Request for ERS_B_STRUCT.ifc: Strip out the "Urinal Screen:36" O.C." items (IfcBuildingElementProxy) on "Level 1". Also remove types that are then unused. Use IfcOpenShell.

First a look at what the model holds.

```python
import ifcopenshell
import ifcopenshell.util.element

model = ifcopenshell.open("ERS_B_STRUCT.ifc")
print(model.schema)
storey = next(s for s in model.by_type("IfcBuildingStorey") if s.Name == "Level 1")
proxies = [e for e in ifcopenshell.util.element.get_decomposition(storey) if e.is_a("IfcBuildingElementProxy")]
seen = {}
for e in proxies:
    element_type = ifcopenshell.util.element.get_type(e)
    name = element_type.Name if element_type not in (None, e) else None
    seen[name] = seen.get(name, 0) + 1
for name, count in sorted(seen.items(), key=str):
    print(count, "x", name)
```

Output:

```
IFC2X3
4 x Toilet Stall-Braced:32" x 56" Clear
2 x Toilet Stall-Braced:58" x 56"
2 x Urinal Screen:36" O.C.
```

```python
import ifcopenshell
import ifcopenshell.api.root
import ifcopenshell.util.element

model = ifcopenshell.open("ERS_B_STRUCT.ifc")

storey = next(s for s in model.by_type("IfcBuildingStorey") if s.Name == "Level 1")
proxies = [e for e in ifcopenshell.util.element.get_decomposition(storey) if e.is_a("IfcBuildingElementProxy")]
targets = [e for e in proxies if (t := ifcopenshell.util.element.get_type(e)) not in (None, e) and t.Name == 'Urinal Screen:36" O.C.']
types = {ifcopenshell.util.element.get_type(e) for e in targets} - {None, *targets}

for e in targets:
    ifcopenshell.api.root.remove_product(model, product=e)
print(len(targets), "removed")

unused = [t for t in types if not ifcopenshell.util.element.get_types(t)]
for t in unused:
    ifcopenshell.api.root.remove_product(model, product=t)
print(len(unused), "unused types removed")

model.write("ERS_B_STRUCT-out.ifc")
```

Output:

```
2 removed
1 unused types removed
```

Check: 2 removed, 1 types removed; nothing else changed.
